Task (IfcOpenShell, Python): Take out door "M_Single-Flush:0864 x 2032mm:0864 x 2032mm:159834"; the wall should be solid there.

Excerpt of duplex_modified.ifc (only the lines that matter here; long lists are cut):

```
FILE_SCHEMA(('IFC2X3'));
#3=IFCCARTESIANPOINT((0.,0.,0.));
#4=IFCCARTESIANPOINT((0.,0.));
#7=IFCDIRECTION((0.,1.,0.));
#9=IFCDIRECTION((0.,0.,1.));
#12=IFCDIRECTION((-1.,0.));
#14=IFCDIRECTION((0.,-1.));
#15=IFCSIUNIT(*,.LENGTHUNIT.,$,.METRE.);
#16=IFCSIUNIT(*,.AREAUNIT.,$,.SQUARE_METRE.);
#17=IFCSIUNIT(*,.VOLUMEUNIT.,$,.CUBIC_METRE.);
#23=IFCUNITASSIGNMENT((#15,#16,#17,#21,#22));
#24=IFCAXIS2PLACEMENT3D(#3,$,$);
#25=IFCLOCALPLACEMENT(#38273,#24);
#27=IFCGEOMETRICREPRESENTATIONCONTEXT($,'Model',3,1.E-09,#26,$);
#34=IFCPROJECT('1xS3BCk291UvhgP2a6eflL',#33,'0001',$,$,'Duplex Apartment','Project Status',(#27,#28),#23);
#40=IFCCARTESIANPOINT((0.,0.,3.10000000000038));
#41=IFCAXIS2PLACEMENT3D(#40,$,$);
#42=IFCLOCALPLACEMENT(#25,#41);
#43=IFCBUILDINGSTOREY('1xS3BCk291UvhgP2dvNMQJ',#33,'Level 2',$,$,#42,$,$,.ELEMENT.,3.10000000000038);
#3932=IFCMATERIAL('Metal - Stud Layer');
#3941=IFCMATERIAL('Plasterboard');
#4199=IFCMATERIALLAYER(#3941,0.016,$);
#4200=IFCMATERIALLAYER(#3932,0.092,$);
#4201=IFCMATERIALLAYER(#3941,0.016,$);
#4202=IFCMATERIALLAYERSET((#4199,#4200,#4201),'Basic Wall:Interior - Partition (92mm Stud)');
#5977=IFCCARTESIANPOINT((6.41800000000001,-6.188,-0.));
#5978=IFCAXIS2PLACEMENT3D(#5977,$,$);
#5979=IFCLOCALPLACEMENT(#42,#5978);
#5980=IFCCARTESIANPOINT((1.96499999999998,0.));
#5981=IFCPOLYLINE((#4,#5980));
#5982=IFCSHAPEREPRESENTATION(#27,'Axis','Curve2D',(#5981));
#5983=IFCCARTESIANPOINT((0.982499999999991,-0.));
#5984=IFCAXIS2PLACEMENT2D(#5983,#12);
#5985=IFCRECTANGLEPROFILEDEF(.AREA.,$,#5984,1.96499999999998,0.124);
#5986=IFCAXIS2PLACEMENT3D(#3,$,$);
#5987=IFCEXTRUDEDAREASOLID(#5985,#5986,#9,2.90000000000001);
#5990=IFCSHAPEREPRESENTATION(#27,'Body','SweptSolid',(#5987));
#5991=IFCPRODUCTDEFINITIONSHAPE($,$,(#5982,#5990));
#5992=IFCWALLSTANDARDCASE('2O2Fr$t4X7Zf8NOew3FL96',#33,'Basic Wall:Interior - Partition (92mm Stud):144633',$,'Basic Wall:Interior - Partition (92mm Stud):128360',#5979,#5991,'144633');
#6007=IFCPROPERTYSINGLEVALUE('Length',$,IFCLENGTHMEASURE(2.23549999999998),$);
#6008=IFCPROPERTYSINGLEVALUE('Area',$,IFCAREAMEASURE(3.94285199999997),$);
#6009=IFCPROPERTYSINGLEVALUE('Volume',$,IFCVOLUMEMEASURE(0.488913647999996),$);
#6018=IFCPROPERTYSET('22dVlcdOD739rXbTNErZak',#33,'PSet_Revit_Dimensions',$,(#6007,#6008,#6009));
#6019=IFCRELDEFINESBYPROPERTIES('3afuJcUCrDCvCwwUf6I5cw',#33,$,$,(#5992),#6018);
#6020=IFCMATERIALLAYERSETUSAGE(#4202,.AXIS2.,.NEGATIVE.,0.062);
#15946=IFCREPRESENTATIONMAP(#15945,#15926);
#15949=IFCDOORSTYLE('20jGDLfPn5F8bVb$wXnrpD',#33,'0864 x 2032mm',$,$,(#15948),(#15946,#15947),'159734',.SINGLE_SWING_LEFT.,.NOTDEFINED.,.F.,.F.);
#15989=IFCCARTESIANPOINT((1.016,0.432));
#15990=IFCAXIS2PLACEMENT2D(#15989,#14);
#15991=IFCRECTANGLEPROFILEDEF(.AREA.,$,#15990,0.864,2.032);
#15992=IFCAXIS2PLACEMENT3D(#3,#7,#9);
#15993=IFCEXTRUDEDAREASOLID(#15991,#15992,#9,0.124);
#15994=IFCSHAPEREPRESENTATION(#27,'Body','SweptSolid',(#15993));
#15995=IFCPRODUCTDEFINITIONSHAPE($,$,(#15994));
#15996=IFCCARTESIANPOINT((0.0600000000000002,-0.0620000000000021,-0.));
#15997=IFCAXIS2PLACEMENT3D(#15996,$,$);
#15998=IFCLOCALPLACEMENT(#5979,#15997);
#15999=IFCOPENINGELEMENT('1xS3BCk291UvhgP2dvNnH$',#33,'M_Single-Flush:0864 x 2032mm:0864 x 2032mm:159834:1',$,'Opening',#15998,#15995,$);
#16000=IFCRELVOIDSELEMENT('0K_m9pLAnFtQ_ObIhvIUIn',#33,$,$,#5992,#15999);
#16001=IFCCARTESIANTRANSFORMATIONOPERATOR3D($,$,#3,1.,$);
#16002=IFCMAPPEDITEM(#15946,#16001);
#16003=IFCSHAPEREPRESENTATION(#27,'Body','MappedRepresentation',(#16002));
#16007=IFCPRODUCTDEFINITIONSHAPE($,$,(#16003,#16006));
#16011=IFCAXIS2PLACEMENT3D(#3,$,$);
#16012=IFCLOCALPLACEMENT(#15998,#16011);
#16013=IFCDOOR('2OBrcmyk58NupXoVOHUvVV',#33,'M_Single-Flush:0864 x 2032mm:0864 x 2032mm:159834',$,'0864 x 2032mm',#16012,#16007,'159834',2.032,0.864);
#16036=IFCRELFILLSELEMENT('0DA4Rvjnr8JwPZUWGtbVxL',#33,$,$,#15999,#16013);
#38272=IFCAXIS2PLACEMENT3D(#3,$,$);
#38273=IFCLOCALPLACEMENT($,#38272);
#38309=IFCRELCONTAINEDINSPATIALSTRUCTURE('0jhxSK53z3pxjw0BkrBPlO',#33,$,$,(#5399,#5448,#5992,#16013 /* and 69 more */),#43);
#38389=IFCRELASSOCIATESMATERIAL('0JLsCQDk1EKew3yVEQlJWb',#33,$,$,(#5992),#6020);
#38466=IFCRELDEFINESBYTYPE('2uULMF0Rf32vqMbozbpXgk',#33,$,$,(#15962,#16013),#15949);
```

```python
import ifcopenshell
import ifcopenshell.api.feature
import ifcopenshell.api.pset
import ifcopenshell.api.root
import ifcopenshell.geom
import ifcopenshell.util.element
import ifcopenshell.util.shape
import ifcopenshell.util.unit

model = ifcopenshell.open("duplex_modified.ifc")
area_scale = ifcopenshell.util.unit.calculate_unit_scale(model, "AREAUNIT")
volume_scale = ifcopenshell.util.unit.calculate_unit_scale(model, "VOLUMEUNIT")
settings = ifcopenshell.geom.settings()


def volume(element):
    """Net volume in cubic metres, openings subtracted."""
    shape = ifcopenshell.geom.create_shape(settings, element)
    return ifcopenshell.util.shape.get_volume(shape.geometry)


door = model.by_guid("2OBrcmyk58NupXoVOHUvVV")
opening = door.FillsVoids[0].RelatingOpeningElement
wall = opening.VoidsElements[0].RelatingBuildingElement
before = volume(wall)

ifcopenshell.api.root.remove_product(model, product=door)
ifcopenshell.api.feature.remove_feature(model, feature=opening)

after = volume(wall)
thickness = 0.124  # wall thickness in metres

# Update the wall's stored quantities.
pset = model.by_id(ifcopenshell.util.element.get_pset(wall, "PSet_Revit_Dimensions", should_inherit=False)["id"])
ifcopenshell.api.pset.edit_pset(model, pset=pset, properties={
    "Area": model.create_entity("IfcAreaMeasure", after / thickness / area_scale),
    "Volume": model.create_entity("IfcVolumeMeasure", after / volume_scale),
})

print(f"wall volume {before:.3f} -> {after:.3f} m3")

model.write("duplex_modified_rev.ifc")
```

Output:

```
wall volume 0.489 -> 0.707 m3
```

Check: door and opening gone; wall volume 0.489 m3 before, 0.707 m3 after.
